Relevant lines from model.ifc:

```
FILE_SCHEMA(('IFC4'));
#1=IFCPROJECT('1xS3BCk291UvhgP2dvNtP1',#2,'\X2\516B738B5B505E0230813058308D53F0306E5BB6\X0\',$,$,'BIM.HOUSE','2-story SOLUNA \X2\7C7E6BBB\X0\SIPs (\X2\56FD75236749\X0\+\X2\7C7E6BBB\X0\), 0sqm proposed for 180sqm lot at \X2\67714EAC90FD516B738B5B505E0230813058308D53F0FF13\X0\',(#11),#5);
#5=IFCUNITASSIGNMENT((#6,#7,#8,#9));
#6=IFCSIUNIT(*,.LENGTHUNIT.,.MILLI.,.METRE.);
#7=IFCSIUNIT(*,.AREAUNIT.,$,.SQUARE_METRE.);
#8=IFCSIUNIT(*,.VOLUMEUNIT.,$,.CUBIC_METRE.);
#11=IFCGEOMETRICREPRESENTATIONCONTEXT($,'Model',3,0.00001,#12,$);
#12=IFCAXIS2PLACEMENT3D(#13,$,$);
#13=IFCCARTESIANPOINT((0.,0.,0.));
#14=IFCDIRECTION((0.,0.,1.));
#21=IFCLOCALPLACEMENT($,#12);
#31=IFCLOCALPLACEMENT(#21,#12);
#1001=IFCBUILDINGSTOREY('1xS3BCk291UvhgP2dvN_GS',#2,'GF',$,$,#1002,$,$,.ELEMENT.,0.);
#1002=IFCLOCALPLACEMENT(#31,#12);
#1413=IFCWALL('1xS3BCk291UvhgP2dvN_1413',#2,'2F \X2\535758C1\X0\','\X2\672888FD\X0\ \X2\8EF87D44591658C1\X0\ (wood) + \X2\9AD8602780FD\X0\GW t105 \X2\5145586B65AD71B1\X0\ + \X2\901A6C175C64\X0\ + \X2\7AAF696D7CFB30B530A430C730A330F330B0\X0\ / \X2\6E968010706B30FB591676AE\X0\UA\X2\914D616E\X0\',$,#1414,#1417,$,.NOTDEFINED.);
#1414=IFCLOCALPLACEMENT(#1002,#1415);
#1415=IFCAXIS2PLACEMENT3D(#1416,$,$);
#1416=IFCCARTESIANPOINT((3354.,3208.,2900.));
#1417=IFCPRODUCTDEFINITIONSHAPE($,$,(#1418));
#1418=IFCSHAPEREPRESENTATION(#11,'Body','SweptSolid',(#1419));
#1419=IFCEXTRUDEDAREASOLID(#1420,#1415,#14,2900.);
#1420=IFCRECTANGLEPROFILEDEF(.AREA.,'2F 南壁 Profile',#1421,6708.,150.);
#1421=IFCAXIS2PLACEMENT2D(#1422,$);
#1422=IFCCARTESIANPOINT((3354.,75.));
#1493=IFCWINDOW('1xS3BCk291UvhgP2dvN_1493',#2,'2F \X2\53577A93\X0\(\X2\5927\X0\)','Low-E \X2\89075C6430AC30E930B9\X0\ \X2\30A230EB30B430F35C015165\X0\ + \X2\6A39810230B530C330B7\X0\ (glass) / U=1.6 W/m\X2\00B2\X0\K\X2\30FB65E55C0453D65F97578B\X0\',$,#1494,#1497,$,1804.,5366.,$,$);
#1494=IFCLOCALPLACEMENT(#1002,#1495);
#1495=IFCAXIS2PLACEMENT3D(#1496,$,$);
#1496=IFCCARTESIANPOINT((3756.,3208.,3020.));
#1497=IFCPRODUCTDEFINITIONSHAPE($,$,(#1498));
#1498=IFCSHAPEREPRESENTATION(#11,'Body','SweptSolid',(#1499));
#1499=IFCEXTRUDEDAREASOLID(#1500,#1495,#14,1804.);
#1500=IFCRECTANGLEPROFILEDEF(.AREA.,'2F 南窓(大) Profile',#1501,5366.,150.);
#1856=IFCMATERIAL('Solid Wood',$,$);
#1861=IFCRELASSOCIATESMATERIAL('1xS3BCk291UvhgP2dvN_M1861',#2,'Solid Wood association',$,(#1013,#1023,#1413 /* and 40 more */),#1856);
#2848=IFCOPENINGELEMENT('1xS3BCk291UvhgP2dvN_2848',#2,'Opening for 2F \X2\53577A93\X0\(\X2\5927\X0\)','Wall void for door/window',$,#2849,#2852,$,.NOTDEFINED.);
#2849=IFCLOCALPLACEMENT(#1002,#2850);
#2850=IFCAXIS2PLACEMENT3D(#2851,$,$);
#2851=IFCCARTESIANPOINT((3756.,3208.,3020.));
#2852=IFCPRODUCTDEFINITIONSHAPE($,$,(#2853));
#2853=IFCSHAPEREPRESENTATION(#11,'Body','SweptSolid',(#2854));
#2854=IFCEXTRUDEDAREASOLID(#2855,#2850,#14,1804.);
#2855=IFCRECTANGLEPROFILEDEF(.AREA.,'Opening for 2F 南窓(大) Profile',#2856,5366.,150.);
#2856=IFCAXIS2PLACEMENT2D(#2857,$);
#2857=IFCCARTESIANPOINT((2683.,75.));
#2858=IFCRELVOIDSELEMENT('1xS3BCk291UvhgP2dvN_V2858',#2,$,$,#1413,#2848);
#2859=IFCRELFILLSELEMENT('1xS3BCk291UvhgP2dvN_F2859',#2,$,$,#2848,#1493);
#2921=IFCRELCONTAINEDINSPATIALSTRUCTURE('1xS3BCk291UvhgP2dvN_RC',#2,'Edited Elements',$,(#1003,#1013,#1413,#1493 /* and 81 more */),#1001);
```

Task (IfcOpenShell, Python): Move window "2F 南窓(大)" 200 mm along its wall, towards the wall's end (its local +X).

```python
import ifcopenshell
import ifcopenshell.api.geometry
import ifcopenshell.util.placement

model = ifcopenshell.open("model.ifc")

window = model.by_id(1493)
opening = window.FillsVoids[0].RelatingOpeningElement
wall = opening.VoidsElements[0].RelatingBuildingElement

wall_matrix = ifcopenshell.util.placement.get_local_placement(wall.ObjectPlacement)
shift = wall_matrix[:3, 0] * 200.0
before = ifcopenshell.util.placement.get_local_placement(window.ObjectPlacement)[:3, 3].copy()

# The window is not placed relative to its opening, so move both.
for product in (opening, window):
    matrix = ifcopenshell.util.placement.get_local_placement(product.ObjectPlacement)
    matrix[:3, 3] += shift
    ifcopenshell.api.geometry.edit_object_placement(model, product=product, matrix=matrix, is_si=False)

after = ifcopenshell.util.placement.get_local_placement(window.ObjectPlacement)[:3, 3]
print("window moved by", (after - before).round(3) + 0.0)

model.write("model-out.ifc")
```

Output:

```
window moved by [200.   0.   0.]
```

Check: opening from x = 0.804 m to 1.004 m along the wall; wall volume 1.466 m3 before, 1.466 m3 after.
